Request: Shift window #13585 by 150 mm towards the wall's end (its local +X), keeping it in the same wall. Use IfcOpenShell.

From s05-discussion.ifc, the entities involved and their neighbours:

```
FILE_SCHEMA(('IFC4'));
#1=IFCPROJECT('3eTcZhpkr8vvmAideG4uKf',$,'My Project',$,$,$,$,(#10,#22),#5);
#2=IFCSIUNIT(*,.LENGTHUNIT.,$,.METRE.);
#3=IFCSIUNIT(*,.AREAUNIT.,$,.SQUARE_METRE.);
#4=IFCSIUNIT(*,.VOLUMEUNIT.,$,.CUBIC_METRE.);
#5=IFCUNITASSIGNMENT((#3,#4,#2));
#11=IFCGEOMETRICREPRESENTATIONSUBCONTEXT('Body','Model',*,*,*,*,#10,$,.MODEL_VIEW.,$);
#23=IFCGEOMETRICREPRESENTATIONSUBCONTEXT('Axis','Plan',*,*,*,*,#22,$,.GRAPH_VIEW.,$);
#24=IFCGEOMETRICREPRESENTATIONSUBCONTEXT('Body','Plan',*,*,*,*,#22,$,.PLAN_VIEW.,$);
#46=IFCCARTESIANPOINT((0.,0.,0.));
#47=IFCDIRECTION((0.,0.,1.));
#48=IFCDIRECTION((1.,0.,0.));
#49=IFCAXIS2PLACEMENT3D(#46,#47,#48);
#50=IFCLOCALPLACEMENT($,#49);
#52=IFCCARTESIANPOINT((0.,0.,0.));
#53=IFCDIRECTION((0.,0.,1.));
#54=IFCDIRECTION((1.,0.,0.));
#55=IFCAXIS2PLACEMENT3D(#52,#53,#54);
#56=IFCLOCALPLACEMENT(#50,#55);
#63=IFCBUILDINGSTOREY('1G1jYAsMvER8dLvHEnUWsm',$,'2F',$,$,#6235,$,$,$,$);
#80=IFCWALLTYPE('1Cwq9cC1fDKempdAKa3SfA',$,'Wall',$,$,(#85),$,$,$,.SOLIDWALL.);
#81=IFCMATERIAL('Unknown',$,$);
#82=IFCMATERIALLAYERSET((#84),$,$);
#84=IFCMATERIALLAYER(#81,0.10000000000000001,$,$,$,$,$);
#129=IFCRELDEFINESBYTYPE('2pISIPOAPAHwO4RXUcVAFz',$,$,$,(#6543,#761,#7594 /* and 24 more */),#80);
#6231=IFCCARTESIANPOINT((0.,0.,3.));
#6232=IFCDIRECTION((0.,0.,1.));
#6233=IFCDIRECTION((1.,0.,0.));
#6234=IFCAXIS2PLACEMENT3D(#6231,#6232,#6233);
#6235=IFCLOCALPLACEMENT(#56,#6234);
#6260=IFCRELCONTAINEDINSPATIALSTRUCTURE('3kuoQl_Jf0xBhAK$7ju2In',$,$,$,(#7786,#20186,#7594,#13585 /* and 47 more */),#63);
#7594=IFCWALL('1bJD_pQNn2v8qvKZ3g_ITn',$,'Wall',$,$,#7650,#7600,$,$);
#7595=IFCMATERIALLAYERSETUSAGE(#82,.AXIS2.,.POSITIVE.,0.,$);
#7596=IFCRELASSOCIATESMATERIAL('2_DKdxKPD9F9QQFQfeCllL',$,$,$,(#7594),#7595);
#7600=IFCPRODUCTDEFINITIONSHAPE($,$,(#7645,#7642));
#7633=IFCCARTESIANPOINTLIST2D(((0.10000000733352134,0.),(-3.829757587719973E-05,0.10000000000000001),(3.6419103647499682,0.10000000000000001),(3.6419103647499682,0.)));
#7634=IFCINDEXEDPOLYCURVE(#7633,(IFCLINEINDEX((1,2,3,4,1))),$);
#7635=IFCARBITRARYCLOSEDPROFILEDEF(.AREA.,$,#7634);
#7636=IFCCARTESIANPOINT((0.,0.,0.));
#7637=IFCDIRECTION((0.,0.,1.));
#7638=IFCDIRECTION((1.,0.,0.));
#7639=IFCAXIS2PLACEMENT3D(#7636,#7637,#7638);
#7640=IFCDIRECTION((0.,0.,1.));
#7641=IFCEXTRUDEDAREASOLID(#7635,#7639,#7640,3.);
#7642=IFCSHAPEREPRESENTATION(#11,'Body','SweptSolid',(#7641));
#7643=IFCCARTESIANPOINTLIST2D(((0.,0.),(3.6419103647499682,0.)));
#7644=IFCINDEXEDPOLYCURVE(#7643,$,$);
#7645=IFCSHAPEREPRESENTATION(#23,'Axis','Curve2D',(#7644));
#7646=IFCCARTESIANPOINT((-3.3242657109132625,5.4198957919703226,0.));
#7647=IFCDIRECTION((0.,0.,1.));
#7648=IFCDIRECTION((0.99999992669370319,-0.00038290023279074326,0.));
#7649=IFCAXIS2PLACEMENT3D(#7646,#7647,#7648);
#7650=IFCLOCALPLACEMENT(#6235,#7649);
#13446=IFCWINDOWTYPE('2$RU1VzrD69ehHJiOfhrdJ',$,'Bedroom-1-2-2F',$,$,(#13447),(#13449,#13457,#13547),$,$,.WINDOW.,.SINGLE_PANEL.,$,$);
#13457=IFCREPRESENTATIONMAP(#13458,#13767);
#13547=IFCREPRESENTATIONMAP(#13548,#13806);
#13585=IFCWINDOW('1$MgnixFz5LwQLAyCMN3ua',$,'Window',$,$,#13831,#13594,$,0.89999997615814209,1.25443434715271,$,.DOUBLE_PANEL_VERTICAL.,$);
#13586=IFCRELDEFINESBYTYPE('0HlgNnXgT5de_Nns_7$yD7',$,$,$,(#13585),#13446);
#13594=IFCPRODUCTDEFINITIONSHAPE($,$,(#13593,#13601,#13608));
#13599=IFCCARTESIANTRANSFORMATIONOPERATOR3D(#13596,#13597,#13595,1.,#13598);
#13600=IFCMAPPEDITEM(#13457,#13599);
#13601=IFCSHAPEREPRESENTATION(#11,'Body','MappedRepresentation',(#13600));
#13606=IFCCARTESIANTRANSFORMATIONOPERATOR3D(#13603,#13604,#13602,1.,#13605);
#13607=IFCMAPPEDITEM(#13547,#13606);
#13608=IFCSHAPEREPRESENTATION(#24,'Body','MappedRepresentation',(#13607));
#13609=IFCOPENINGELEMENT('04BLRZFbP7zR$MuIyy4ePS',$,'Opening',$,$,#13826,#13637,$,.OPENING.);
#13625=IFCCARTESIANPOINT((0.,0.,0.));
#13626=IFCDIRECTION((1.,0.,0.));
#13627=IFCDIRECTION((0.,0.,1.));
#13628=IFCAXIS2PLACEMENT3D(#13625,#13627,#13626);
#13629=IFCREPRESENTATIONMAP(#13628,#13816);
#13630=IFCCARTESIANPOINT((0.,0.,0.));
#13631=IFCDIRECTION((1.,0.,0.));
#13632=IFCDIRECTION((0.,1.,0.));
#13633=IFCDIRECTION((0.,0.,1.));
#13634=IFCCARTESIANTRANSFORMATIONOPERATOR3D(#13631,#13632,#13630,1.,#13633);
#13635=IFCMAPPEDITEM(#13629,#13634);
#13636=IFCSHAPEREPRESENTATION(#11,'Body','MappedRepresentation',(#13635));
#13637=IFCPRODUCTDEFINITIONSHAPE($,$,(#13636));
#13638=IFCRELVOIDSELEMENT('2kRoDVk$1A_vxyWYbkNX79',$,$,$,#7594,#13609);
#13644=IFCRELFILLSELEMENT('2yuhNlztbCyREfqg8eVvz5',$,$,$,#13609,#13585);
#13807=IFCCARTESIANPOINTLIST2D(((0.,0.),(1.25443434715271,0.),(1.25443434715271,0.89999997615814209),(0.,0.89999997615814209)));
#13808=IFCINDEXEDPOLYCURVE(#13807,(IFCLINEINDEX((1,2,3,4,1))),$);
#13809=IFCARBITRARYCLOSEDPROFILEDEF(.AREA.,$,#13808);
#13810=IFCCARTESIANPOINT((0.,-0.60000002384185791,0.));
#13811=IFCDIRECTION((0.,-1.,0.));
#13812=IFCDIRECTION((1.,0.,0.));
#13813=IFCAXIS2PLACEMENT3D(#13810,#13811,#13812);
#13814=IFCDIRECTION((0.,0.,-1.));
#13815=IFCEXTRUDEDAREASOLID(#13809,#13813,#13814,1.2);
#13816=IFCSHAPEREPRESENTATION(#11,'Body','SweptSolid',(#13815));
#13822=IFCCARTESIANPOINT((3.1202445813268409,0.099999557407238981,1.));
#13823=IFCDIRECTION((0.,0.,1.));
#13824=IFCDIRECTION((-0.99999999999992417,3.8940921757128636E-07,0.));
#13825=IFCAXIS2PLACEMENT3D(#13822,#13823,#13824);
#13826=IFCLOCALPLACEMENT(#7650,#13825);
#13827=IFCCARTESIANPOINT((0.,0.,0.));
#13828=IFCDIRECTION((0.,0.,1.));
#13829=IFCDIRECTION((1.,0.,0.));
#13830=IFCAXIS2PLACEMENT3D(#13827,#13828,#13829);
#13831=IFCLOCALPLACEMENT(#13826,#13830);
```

```python
import ifcopenshell
import ifcopenshell.api.geometry
import ifcopenshell.util.placement
import ifcopenshell.util.unit

model = ifcopenshell.open("s05-discussion.ifc")
unit_scale = ifcopenshell.util.unit.calculate_unit_scale(model)

window = model.by_guid("1$MgnixFz5LwQLAyCMN3ua")
opening = window.FillsVoids[0].RelatingOpeningElement
wall = opening.VoidsElements[0].RelatingBuildingElement

wall_matrix = ifcopenshell.util.placement.get_local_placement(wall.ObjectPlacement)
shift = wall_matrix[:3, 0] * 0.15 / unit_scale
before = ifcopenshell.util.placement.get_local_placement(window.ObjectPlacement)[:3, 3].copy()

# The window is placed relative to its opening, so it follows when the opening moves.
matrix = ifcopenshell.util.placement.get_local_placement(opening.ObjectPlacement)
matrix[:3, 3] += shift
ifcopenshell.api.geometry.edit_object_placement(
    model, product=opening, matrix=matrix, is_si=False, should_transform_children=True
)

after = ifcopenshell.util.placement.get_local_placement(window.ObjectPlacement)[:3, 3]
print("window moved by", (after - before).round(3) + 0.0)

model.write("s05-discussion_rev.ifc")
```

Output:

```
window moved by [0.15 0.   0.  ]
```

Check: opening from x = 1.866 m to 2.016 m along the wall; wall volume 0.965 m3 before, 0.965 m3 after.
